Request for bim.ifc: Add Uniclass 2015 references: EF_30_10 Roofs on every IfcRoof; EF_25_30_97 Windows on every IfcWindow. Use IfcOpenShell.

First a look at what the model holds.

```python
import ifcopenshell

model = ifcopenshell.open("bim.ifc")
print(model.schema)
print("classifications:", [c.Name for c in model.by_type("IfcClassification")])
for ifc_class in ("IfcDoor", "IfcRoof", "IfcStair", "IfcWall", "IfcWindow"):
    print(ifc_class, len(model.by_type(ifc_class)))
```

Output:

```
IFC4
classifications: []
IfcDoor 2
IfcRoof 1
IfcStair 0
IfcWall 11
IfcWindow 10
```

```python
import ifcopenshell
import ifcopenshell.api.classification

model = ifcopenshell.open("bim.ifc")

system = ifcopenshell.api.classification.add_classification(model, classification="Uniclass 2015")

codes = {
    "IfcRoof": ("EF_30_10", "Roofs"),
    "IfcWindow": ("EF_25_30_97", "Windows"),
}
for ifc_class, (code, name) in codes.items():
    products = model.by_type(ifc_class)
    ifcopenshell.api.classification.add_reference(
        model, products=products, classification=system, identification=code, name=name
    )
    print(code, len(products))

model.write("bim-out.ifc")
```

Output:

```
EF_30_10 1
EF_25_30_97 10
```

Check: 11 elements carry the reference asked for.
